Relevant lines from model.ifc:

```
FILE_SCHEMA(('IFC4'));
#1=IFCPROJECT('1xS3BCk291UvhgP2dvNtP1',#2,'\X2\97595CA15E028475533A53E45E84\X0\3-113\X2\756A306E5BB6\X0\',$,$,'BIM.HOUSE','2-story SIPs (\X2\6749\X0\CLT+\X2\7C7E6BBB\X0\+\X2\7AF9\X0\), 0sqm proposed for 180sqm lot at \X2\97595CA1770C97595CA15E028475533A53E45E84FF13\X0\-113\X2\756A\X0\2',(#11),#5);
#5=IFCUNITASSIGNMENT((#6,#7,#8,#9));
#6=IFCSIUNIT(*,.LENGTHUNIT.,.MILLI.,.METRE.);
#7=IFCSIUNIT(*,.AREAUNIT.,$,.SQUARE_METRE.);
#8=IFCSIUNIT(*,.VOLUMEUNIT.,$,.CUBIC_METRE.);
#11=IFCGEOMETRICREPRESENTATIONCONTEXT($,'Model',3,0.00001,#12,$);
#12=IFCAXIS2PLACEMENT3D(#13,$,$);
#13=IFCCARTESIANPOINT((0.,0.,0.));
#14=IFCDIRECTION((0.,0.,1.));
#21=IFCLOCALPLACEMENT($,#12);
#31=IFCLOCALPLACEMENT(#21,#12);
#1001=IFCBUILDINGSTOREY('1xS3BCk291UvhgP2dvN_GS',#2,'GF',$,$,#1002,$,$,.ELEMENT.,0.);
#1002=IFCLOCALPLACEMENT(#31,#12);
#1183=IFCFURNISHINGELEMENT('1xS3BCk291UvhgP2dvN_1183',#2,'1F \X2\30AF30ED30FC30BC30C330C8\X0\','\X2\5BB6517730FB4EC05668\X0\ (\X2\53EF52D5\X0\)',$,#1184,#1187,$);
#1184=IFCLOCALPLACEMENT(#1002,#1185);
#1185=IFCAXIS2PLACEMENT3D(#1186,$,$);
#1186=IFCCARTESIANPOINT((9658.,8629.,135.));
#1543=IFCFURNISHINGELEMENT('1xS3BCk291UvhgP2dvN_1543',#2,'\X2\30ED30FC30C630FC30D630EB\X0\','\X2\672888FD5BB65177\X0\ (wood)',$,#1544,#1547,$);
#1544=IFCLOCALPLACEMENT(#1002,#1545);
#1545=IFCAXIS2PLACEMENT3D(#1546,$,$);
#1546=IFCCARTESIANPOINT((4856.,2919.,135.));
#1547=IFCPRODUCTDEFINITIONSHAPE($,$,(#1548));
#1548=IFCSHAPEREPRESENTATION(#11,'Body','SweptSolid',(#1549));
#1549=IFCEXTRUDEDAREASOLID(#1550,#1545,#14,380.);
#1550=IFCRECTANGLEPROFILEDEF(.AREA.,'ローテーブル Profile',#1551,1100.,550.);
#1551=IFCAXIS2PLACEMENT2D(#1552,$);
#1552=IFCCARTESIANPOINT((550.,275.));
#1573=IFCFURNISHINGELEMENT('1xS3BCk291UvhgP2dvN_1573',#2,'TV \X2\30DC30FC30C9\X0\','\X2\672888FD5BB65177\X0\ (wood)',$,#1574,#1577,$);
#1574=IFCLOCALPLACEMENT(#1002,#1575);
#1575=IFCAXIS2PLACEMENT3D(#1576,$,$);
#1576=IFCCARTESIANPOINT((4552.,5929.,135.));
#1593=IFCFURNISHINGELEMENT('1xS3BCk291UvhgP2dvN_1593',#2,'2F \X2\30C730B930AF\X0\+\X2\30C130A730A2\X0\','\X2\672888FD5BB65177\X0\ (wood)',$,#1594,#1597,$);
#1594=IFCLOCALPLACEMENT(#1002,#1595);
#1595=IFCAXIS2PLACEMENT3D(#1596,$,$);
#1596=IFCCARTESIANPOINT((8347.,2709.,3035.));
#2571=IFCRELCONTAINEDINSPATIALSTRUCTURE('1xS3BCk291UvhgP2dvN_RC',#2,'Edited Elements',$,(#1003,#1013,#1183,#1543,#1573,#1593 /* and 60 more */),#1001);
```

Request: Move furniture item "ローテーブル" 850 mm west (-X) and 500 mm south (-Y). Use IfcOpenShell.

```python
import ifcopenshell
import ifcopenshell.api.geometry
import ifcopenshell.util.placement
import ifcopenshell.util.unit

model = ifcopenshell.open("model.ifc")
unit_scale = ifcopenshell.util.unit.calculate_unit_scale(model)

item = model.by_guid("1xS3BCk291UvhgP2dvN_1543")
matrix = ifcopenshell.util.placement.get_local_placement(item.ObjectPlacement)
matrix[0, 3] -= 0.85 / unit_scale
matrix[1, 3] -= 0.5 / unit_scale
ifcopenshell.api.geometry.edit_object_placement(model, product=item, matrix=matrix, is_si=False)

print(ifcopenshell.util.placement.get_local_placement(item.ObjectPlacement).round(3) + 0.0)

model.write("model_edited.ifc")
```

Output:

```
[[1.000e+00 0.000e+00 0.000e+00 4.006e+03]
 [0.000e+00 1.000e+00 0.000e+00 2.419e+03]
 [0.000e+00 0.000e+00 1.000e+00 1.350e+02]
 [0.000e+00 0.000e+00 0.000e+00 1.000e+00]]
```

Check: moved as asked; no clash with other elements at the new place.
